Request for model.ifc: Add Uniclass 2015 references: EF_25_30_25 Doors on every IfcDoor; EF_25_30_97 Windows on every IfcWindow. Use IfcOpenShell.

First a look at what the model holds.

```python
import ifcopenshell

model = ifcopenshell.open("model.ifc")
print(model.schema)
print("classifications:", [c.Name for c in model.by_type("IfcClassification")])
for ifc_class in ("IfcDoor", "IfcRoof", "IfcStair", "IfcWall", "IfcWindow"):
    print(ifc_class, len(model.by_type(ifc_class)))
```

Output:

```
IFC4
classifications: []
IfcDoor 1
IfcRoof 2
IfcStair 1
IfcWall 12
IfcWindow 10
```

```python
import ifcopenshell
import ifcopenshell.api.classification

model = ifcopenshell.open("model.ifc")

system = ifcopenshell.api.classification.add_classification(model, classification="Uniclass 2015")

codes = {
    "IfcDoor": ("EF_25_30_25", "Doors"),
    "IfcWindow": ("EF_25_30_97", "Windows"),
}
for ifc_class, (code, name) in codes.items():
    products = model.by_type(ifc_class)
    ifcopenshell.api.classification.add_reference(
        model, products=products, classification=system, identification=code, name=name
    )
    print(code, len(products))

model.write("model_rev.ifc")
```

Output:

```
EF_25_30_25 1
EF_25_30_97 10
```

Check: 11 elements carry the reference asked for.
